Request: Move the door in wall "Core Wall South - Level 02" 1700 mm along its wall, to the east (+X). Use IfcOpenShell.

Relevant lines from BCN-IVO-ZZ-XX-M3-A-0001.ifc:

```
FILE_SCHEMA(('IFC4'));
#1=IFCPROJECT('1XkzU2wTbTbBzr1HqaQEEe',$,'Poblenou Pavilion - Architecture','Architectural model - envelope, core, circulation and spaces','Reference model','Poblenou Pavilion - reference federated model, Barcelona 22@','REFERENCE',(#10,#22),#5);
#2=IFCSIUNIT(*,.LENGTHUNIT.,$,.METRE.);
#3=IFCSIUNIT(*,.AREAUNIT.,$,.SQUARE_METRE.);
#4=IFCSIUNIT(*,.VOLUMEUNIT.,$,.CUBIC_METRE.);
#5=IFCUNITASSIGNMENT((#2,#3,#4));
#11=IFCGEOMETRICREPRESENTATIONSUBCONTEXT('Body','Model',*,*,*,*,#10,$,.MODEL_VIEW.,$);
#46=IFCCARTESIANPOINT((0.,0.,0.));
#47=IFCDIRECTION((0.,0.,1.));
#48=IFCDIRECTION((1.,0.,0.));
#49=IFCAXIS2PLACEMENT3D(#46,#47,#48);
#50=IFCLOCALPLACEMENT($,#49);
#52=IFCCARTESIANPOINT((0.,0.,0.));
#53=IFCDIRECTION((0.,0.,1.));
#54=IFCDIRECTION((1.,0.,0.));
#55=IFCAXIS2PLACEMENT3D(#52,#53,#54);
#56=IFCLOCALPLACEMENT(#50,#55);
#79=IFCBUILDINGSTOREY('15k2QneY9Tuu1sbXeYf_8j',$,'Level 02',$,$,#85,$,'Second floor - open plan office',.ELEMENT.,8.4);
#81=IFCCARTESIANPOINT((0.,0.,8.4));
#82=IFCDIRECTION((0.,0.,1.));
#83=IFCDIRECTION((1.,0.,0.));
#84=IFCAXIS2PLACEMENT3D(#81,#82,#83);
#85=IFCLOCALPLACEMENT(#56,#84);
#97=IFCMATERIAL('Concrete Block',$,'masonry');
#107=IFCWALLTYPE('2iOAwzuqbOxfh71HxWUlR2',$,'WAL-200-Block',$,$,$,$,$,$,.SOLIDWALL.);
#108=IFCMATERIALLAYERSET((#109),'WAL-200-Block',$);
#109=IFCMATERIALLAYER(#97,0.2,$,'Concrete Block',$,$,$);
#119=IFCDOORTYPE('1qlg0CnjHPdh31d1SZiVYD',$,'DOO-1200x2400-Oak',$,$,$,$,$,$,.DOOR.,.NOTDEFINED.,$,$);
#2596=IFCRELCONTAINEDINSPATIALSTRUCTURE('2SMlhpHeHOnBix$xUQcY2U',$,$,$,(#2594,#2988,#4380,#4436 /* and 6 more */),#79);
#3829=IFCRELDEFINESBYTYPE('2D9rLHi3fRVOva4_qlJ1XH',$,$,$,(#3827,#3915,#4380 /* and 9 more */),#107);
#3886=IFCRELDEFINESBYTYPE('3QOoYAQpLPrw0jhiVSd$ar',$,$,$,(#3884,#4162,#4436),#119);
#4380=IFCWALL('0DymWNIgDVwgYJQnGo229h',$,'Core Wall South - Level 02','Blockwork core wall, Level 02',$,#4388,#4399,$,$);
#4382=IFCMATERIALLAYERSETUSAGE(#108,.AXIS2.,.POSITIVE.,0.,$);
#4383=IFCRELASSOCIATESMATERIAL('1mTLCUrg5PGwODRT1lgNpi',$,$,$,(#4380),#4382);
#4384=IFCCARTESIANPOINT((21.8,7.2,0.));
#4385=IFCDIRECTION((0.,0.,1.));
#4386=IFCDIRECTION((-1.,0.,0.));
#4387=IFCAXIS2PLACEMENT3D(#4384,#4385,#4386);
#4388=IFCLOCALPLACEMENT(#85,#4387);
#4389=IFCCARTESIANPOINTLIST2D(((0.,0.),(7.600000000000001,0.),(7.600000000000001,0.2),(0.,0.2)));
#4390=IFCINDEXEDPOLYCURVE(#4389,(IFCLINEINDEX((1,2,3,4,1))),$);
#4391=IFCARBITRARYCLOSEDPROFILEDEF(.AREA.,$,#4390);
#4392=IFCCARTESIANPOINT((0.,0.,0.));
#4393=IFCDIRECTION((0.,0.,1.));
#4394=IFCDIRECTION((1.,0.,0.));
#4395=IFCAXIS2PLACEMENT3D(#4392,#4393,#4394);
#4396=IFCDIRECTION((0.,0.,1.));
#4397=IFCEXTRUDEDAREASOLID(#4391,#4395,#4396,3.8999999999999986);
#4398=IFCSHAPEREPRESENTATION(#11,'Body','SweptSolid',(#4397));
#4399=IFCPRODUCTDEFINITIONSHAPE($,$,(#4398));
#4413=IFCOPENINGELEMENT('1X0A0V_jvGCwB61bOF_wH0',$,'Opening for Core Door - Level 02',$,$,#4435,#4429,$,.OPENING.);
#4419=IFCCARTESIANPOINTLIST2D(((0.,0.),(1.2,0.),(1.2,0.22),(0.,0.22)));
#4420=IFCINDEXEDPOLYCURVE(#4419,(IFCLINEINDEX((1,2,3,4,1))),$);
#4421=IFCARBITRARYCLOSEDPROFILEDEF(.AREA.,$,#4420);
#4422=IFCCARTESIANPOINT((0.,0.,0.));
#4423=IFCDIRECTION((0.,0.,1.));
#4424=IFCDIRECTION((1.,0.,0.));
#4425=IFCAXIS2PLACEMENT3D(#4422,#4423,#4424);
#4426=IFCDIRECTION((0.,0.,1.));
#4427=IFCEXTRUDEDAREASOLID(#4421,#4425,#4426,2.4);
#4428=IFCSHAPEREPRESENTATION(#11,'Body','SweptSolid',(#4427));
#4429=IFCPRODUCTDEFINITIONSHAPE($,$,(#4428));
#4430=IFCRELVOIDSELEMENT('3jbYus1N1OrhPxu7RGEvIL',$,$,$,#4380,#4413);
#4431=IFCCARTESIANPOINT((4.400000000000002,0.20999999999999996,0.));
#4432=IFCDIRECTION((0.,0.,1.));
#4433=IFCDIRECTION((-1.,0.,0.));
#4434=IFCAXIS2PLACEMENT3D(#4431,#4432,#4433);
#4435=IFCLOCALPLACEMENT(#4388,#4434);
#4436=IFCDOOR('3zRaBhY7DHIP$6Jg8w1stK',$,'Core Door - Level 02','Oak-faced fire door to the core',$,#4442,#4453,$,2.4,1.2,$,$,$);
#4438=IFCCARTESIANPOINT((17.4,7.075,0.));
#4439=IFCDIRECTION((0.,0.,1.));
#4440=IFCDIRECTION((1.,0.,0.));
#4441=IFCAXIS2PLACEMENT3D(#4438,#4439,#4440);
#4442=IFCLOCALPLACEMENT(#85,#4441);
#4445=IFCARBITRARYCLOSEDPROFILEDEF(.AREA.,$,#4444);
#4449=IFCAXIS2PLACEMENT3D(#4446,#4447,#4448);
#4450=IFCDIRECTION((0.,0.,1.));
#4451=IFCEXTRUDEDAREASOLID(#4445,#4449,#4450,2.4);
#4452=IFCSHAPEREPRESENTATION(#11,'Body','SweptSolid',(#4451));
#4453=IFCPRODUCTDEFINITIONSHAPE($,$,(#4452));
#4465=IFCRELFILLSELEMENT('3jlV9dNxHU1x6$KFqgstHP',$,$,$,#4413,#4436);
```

```python
import ifcopenshell
import ifcopenshell.api.geometry
import ifcopenshell.util.placement
import ifcopenshell.util.unit

model = ifcopenshell.open("BCN-IVO-ZZ-XX-M3-A-0001.ifc")
unit_scale = ifcopenshell.util.unit.calculate_unit_scale(model)

door = model.by_id(4436)
opening = door.FillsVoids[0].RelatingOpeningElement
wall = opening.VoidsElements[0].RelatingBuildingElement

wall_matrix = ifcopenshell.util.placement.get_local_placement(wall.ObjectPlacement)
shift = wall_matrix[:3, 0] * -1.7 / unit_scale
before = ifcopenshell.util.placement.get_local_placement(door.ObjectPlacement)[:3, 3].copy()

# The door is not placed relative to its opening, so move both.
for product in (opening, door):
    matrix = ifcopenshell.util.placement.get_local_placement(product.ObjectPlacement)
    matrix[:3, 3] += shift
    ifcopenshell.api.geometry.edit_object_placement(model, product=product, matrix=matrix, is_si=False)

after = ifcopenshell.util.placement.get_local_placement(door.ObjectPlacement)[:3, 3]
print("door moved by", (after - before).round(3) + 0.0)

model.write("BCN-IVO-ZZ-XX-M3-A-0001_updated.ifc")
```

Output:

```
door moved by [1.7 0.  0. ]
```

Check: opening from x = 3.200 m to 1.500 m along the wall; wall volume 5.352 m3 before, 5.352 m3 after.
